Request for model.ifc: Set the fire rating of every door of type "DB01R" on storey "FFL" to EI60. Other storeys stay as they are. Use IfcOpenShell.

First a look at what the model holds.

```python
import ifcopenshell
import ifcopenshell.util.element

model = ifcopenshell.open("model.ifc")
print(model.schema)
storey = next(s for s in model.by_type("IfcBuildingStorey") if s.Name == "FFL")
doors = [e for e in ifcopenshell.util.element.get_decomposition(storey) if e.is_a("IfcDoor")]
seen = {}
for e in doors:
    element_type = ifcopenshell.util.element.get_type(e)
    key = (element_type.Name if element_type != e and element_type else None, ifcopenshell.util.element.get_pset(e, "Pset_DoorCommon", "FireRating"))
    seen[key] = seen.get(key, 0) + 1
for (name, value), count in sorted(seen.items(), key=str):
    print(count, "x", name, "|", value)
```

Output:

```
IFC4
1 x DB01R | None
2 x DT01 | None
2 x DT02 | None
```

```python
import ifcopenshell
import ifcopenshell.api.pset
import ifcopenshell.util.element

model = ifcopenshell.open("model.ifc")

storey = next(s for s in model.by_type("IfcBuildingStorey") if s.Name == "FFL")
doors = [e for e in ifcopenshell.util.element.get_decomposition(storey) if e.is_a("IfcDoor")]

count = 0
for e in doors:
    element_type = ifcopenshell.util.element.get_type(e)
    if element_type in (None, e) or element_type.Name != "DB01R":
        continue
    # add_pset returns the element's existing set when there is one.
    pset = ifcopenshell.api.pset.add_pset(model, product=e, name="Pset_DoorCommon")
    ifcopenshell.api.pset.edit_pset(model, pset=pset, properties={"FireRating": "EI60"})
    count += 1

print(count, "doors updated")

model.write("model_v2.ifc")
```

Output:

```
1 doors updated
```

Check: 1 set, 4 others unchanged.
